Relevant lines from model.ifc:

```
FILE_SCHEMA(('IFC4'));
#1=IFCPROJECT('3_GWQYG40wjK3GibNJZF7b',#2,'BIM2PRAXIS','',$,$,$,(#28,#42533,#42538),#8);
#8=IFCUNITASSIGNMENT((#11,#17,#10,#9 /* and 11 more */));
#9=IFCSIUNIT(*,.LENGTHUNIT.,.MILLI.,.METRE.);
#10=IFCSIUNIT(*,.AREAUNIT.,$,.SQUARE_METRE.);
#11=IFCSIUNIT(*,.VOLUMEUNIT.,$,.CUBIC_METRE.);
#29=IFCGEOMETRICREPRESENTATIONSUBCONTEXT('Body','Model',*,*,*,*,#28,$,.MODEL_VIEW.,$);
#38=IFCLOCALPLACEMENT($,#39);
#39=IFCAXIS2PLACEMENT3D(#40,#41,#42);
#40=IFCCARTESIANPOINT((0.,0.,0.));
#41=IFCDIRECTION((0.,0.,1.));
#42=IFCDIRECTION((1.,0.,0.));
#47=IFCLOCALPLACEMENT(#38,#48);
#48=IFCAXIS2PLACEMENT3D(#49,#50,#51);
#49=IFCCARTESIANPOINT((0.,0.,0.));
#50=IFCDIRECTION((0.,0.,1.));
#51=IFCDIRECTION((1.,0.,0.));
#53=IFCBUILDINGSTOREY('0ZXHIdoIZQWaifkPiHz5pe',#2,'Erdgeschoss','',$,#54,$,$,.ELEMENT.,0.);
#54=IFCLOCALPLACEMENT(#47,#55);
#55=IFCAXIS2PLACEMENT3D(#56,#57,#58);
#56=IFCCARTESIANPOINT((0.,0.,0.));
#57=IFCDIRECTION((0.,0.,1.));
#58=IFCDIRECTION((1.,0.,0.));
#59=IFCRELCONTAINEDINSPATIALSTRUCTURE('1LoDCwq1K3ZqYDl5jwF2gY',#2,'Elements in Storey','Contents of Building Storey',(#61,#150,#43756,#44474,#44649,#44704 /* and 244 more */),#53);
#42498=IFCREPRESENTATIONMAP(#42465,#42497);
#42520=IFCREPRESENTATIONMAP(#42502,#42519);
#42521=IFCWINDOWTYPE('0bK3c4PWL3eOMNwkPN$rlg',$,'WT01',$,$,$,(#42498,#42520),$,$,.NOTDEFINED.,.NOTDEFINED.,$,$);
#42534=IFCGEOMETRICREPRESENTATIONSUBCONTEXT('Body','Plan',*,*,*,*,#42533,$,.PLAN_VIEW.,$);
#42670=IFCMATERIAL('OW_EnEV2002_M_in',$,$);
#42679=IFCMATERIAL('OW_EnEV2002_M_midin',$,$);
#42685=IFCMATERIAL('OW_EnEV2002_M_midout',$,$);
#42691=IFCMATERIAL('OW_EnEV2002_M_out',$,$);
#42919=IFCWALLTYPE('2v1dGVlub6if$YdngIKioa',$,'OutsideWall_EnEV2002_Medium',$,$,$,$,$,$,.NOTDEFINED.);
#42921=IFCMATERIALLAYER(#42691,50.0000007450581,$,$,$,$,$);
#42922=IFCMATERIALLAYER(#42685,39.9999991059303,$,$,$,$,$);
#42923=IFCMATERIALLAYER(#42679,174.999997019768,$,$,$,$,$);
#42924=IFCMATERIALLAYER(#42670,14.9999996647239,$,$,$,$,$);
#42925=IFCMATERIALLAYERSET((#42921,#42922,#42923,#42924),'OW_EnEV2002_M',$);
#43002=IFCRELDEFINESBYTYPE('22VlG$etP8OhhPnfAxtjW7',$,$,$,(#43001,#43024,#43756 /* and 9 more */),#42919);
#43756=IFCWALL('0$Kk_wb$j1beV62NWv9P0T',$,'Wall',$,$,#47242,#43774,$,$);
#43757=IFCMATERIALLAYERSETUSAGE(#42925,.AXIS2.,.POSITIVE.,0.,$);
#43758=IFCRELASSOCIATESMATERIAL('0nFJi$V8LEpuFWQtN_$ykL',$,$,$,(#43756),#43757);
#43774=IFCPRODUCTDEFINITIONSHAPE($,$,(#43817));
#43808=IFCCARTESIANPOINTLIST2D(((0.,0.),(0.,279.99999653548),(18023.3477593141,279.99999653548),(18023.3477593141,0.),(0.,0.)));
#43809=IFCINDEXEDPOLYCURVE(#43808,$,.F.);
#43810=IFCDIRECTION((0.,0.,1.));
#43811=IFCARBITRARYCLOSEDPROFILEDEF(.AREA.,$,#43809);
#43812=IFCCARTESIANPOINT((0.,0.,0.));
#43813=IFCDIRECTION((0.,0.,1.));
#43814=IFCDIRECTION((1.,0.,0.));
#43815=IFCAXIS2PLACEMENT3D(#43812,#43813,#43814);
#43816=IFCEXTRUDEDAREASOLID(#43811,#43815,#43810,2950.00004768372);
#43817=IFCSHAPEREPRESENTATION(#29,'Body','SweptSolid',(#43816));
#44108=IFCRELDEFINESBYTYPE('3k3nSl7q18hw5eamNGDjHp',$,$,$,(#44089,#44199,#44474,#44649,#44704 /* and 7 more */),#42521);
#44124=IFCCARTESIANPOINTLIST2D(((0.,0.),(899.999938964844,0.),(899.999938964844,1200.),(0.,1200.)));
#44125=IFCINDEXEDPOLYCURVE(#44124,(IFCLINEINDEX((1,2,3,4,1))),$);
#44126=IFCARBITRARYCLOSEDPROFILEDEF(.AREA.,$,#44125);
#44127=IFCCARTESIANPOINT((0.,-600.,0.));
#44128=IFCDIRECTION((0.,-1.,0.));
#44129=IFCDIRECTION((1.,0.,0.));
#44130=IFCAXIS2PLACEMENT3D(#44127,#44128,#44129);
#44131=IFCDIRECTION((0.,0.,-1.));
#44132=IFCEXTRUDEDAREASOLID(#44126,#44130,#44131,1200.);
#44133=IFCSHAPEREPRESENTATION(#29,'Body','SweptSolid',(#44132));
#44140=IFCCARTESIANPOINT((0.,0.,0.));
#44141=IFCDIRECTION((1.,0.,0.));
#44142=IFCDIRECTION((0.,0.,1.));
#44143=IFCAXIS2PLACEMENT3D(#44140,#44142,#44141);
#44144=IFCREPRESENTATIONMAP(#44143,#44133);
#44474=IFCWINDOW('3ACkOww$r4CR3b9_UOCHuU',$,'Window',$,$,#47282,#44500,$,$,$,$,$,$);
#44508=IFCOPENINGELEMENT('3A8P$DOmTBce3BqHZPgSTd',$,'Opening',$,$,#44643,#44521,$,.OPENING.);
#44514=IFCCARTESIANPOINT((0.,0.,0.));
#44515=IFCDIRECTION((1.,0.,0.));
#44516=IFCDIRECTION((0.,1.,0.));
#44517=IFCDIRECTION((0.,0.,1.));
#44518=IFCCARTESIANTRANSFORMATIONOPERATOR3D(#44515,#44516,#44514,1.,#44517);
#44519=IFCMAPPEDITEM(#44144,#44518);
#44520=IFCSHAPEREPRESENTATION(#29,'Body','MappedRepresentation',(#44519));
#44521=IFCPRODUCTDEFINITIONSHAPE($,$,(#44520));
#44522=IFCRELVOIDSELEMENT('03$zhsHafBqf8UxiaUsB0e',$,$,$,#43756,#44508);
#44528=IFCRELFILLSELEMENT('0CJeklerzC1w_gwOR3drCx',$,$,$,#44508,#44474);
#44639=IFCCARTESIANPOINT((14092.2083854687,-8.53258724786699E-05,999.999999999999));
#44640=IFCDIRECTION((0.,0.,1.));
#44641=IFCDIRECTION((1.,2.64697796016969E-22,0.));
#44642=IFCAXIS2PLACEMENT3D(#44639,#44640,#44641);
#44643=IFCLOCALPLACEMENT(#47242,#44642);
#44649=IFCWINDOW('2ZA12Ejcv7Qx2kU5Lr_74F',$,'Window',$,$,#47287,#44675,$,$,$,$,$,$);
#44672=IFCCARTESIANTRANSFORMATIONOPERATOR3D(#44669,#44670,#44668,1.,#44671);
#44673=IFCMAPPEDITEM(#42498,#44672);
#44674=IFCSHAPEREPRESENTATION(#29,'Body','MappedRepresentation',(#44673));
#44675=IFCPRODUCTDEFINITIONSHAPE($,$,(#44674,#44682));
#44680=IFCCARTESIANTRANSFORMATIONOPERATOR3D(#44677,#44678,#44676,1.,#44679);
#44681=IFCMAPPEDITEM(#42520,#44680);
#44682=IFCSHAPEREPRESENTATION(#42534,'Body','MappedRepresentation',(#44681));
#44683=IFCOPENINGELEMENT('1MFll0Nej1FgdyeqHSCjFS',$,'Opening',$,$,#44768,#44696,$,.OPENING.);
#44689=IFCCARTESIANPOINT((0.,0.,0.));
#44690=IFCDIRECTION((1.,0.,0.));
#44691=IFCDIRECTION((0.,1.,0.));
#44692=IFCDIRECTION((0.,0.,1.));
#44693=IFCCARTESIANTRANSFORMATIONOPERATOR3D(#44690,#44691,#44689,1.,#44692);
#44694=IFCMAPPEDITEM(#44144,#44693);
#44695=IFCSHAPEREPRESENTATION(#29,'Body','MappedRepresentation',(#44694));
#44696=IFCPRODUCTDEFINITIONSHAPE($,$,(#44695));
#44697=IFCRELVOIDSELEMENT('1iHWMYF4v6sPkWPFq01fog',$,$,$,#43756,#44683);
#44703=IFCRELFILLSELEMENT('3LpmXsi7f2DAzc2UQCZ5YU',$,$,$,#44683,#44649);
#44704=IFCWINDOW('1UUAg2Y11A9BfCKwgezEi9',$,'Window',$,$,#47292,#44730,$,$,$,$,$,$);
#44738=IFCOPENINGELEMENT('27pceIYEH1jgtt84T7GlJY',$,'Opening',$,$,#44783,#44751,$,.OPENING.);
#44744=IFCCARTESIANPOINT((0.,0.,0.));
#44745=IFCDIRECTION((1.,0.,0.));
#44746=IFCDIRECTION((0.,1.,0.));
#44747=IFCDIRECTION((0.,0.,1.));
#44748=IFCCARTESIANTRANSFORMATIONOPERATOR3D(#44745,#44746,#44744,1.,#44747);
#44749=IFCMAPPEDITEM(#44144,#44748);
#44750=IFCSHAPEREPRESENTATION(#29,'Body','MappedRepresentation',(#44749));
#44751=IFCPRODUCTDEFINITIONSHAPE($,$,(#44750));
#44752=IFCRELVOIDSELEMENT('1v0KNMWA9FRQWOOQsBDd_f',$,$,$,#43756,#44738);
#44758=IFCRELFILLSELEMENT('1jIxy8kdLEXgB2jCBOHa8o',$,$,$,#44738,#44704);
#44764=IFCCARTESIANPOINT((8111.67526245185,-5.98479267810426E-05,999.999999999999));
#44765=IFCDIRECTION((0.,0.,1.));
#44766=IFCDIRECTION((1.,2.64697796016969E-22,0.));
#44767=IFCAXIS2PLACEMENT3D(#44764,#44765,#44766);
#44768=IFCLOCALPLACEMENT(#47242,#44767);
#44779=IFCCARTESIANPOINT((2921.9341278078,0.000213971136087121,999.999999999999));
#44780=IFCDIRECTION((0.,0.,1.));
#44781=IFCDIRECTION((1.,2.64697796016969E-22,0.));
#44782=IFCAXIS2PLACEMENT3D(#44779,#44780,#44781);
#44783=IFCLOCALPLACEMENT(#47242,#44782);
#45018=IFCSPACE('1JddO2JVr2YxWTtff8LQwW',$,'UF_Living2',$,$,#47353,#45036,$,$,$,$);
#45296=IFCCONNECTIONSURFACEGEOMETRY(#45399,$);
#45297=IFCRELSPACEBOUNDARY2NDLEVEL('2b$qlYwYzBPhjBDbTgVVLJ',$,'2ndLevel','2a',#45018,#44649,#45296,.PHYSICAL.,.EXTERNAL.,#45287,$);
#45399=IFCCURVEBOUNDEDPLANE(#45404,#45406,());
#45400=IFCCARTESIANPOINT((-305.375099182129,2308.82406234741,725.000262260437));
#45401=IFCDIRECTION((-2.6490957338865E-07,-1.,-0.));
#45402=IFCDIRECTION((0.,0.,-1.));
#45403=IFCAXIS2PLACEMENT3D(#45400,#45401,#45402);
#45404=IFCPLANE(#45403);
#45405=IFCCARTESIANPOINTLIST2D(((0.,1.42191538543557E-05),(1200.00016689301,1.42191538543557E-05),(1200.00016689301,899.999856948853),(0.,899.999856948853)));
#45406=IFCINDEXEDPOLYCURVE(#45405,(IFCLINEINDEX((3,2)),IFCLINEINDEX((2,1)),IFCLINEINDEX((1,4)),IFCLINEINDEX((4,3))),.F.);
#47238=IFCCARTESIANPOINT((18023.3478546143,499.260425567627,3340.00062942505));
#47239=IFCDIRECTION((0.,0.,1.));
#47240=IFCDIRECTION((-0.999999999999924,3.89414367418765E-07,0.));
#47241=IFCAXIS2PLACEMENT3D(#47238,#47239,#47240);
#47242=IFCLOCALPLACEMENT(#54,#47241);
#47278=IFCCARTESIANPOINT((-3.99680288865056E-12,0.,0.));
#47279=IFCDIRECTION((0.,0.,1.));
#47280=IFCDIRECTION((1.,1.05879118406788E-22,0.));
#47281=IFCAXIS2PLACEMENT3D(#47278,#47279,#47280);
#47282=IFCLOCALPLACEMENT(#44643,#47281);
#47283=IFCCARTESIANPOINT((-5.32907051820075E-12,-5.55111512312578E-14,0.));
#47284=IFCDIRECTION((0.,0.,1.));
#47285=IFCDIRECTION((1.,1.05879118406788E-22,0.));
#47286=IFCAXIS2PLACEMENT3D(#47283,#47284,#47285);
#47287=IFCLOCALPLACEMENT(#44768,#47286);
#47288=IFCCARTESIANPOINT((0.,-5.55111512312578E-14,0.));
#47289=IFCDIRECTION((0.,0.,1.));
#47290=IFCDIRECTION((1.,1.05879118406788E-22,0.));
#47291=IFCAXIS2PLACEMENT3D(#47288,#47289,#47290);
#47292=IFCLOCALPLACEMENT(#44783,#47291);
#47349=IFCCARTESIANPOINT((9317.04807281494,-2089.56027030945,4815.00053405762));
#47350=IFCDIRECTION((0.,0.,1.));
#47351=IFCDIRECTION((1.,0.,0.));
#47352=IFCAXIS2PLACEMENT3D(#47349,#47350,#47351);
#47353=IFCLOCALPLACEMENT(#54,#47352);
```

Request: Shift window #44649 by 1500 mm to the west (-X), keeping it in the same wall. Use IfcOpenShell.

```python
import numpy as np
import ifcopenshell
import ifcopenshell.api.geometry
import ifcopenshell.util.placement
import ifcopenshell.util.unit

model = ifcopenshell.open("model.ifc")
unit_scale = ifcopenshell.util.unit.calculate_unit_scale(model)

window = model.by_guid("2ZA12Ejcv7Qx2kU5Lr_74F")
opening = window.FillsVoids[0].RelatingOpeningElement
wall = opening.VoidsElements[0].RelatingBuildingElement

wall_matrix = ifcopenshell.util.placement.get_local_placement(wall.ObjectPlacement)
shift = wall_matrix[:3, 0] * 1.5 / unit_scale
before = ifcopenshell.util.placement.get_local_placement(window.ObjectPlacement)[:3, 3].copy()

# The window is placed relative to its opening, so it follows when the opening moves.
matrix = ifcopenshell.util.placement.get_local_placement(opening.ObjectPlacement)
matrix[:3, 3] += shift
ifcopenshell.api.geometry.edit_object_placement(
    model, product=opening, matrix=matrix, is_si=False, should_transform_children=True
)

# Space boundary surfaces are stored in each space's coordinates; move them too.
for rel in window.ProvidesBoundaries:
    if not rel.ConnectionGeometry:
        continue
    surface = rel.ConnectionGeometry.SurfaceOnRelatingElement.BasisSurface
    space_matrix = ifcopenshell.util.placement.get_local_placement(rel.RelatingSpace.ObjectPlacement)
    point = np.array(surface.Position.Location.Coordinates) + space_matrix[:3, :3].T @ shift
    surface.Position = model.createIfcAxis2Placement3D(
        model.createIfcCartesianPoint(point.tolist()), surface.Position.Axis, surface.Position.RefDirection
    )

after = ifcopenshell.util.placement.get_local_placement(window.ObjectPlacement)[:3, 3]
print("window moved by", (after - before).round(3) + 0.0)

model.write("model_updated.ifc")
```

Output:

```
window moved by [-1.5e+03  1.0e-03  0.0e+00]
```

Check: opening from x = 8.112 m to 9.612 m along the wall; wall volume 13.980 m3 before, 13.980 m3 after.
